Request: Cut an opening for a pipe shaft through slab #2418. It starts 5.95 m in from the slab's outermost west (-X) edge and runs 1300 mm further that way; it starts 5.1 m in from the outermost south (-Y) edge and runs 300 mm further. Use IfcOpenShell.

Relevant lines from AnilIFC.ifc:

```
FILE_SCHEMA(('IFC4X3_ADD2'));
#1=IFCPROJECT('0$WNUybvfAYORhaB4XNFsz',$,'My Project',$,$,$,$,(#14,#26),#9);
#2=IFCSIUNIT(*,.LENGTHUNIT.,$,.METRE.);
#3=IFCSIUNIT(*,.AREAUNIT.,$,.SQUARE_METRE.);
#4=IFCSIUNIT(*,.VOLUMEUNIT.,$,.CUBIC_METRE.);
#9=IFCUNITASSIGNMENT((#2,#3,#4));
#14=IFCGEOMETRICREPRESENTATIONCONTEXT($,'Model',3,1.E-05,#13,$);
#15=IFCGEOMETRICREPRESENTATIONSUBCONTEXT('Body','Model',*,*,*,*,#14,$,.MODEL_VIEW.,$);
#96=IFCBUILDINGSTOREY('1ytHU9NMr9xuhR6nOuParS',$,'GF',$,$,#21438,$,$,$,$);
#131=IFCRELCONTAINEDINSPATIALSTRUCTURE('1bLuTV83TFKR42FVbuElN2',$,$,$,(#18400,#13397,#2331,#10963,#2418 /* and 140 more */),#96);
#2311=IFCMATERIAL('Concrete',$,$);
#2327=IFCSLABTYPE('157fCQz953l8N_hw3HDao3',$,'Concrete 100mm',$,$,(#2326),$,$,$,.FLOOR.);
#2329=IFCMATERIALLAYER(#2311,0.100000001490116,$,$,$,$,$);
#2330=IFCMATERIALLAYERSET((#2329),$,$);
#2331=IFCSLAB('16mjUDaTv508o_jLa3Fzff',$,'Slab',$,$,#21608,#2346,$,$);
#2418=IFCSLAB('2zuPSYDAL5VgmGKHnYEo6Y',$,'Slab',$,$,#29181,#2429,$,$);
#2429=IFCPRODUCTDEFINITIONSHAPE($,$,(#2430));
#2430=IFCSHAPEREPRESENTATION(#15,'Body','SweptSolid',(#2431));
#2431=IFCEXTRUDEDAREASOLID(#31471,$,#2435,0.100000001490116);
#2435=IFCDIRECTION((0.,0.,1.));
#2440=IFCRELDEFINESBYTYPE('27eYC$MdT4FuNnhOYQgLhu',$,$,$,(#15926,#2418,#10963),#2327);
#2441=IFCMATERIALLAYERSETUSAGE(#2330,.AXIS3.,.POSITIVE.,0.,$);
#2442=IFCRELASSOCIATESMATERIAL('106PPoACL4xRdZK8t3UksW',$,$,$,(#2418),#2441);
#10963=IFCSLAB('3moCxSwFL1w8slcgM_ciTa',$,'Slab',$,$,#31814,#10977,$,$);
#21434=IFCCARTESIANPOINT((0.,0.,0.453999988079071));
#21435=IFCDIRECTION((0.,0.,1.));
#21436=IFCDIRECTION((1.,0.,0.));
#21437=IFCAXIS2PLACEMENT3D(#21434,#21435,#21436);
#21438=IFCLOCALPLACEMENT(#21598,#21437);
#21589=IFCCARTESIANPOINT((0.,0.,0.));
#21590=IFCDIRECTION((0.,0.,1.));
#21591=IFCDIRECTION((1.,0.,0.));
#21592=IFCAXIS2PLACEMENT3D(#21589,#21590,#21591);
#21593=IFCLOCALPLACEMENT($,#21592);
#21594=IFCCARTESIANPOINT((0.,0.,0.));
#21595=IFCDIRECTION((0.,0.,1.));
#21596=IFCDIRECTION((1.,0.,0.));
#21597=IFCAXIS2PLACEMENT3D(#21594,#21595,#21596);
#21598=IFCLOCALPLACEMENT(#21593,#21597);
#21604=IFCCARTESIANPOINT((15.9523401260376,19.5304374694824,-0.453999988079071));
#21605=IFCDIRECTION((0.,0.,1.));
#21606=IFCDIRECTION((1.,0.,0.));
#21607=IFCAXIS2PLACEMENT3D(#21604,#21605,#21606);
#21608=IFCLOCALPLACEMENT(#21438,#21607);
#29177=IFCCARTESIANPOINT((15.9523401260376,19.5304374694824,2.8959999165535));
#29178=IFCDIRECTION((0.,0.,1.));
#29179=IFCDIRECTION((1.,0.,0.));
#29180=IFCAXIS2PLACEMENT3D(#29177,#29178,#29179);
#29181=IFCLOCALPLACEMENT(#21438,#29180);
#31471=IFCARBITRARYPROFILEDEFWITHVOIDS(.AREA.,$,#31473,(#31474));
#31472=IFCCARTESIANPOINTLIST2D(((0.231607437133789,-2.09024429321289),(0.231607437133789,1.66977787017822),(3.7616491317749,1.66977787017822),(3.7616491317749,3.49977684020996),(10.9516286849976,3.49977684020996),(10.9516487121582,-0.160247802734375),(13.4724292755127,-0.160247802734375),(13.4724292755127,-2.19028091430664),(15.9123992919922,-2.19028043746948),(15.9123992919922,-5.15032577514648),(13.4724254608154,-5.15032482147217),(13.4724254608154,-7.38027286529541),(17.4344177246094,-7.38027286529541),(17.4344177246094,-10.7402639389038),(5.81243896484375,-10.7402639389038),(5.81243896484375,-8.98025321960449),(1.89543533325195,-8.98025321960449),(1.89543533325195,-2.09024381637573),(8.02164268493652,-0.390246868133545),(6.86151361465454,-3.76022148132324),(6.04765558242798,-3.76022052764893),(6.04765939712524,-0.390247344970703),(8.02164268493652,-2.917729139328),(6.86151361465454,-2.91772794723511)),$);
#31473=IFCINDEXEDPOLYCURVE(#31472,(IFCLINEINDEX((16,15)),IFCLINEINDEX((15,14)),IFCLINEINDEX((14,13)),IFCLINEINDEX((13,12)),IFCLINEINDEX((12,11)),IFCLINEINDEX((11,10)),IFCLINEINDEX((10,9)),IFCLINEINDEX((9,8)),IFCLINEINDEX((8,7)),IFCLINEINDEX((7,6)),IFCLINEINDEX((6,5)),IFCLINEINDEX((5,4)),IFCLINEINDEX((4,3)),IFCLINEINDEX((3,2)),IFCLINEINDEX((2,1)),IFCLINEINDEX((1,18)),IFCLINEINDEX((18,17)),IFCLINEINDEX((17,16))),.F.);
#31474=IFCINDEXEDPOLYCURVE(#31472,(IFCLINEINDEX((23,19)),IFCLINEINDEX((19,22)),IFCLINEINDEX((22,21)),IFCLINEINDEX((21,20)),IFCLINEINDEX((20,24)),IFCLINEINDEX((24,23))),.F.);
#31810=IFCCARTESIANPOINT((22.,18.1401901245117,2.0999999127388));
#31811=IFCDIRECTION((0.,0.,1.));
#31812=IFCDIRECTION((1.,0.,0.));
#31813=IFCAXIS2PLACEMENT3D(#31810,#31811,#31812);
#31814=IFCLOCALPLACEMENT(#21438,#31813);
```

```python
import numpy as np
import ifcopenshell
import ifcopenshell.api.feature
import ifcopenshell.api.geometry
import ifcopenshell.api.root
import ifcopenshell.geom
import ifcopenshell.util.placement
import ifcopenshell.util.representation
import ifcopenshell.util.shape
import ifcopenshell.util.unit

model = ifcopenshell.open("AnilIFC.ifc")
unit_scale = ifcopenshell.util.unit.calculate_unit_scale(model)
settings = ifcopenshell.geom.settings()


def volume(element):
    """Net volume in cubic metres, openings subtracted."""
    shape = ifcopenshell.geom.create_shape(settings, element)
    return ifcopenshell.util.shape.get_volume(shape.geometry)


slab = model.by_id(2418)
before = volume(slab)

# Extent in the slab's own axes, in metres. The edges named are its -X and -Y sides.
slab_shape = ifcopenshell.geom.create_shape(settings, slab)
vertices = ifcopenshell.util.shape.get_vertices(slab_shape.geometry)
x_min, y_min, bottom = vertices.min(axis=0)
top = vertices[:, 2].max()

opening = ifcopenshell.api.root.create_entity(model, ifc_class="IfcOpeningElement", name="Pipe shaft opening", predefined_type="OPENING")
context = ifcopenshell.util.representation.get_context(model, "Model", "Body", "MODEL_VIEW")
width, depth = 1.3, 0.3
outline = [(0.0, 0.0), (width, 0.0), (width, depth), (0.0, depth), (0.0, 0.0)]
# Overshoot both faces by 50 mm so the cut is clean.
shape = ifcopenshell.api.geometry.add_slab_representation(
    model, context=context, depth=top - bottom + 0.1, polyline=outline
)
ifcopenshell.api.geometry.assign_representation(model, product=opening, representation=shape)

matrix = ifcopenshell.util.placement.get_local_placement(slab.ObjectPlacement)
matrix[:, 3] = matrix @ np.append(np.array([x_min + 5.95, y_min + 5.1, bottom - 0.05]) / unit_scale, 1.0)
ifcopenshell.api.geometry.edit_object_placement(model, product=opening, matrix=matrix, is_si=False)
ifcopenshell.api.feature.add_feature(model, feature=opening, element=slab)

after = volume(slab)

print(f"slab volume {before:.3f} -> {after:.3f} m3")

model.write("AnilIFC_updated.ifc")
```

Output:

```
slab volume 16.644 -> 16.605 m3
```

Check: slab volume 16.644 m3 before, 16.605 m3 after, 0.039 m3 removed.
